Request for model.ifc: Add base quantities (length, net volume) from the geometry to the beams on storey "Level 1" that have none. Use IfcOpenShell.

First a look at what the model holds.

```python
import ifcopenshell
import ifcopenshell.util.element
import ifcopenshell.util.unit

model = ifcopenshell.open("model.ifc")
print(model.schema)
for unit_type in ("LENGTHUNIT", "AREAUNIT", "VOLUMEUNIT"):
    print(unit_type, ifcopenshell.util.unit.calculate_unit_scale(model, unit_type))
storey = next(s for s in model.by_type("IfcBuildingStorey") if s.Name == "Level 1")
beams = [e for e in ifcopenshell.util.element.get_decomposition(storey) if e.is_a("IfcBeam")]
for e in sorted(beams, key=lambda e: e.id()):
    print(e.id(), e.is_a(), e.Name, list(ifcopenshell.util.element.get_psets(e, qtos_only=True)), sep=" | ")
```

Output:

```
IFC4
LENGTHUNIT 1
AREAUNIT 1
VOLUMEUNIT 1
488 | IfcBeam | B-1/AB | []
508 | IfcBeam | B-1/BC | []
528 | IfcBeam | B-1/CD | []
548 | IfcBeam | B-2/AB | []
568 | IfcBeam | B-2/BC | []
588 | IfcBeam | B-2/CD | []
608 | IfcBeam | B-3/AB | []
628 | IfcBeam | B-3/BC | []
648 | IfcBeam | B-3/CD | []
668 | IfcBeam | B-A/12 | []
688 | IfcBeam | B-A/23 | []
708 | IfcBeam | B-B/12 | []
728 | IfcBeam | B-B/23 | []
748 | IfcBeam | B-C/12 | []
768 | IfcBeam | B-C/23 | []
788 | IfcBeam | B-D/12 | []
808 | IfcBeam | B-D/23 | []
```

```python
import ifcopenshell
import ifcopenshell.api.pset
import ifcopenshell.geom
import ifcopenshell.util.element
import ifcopenshell.util.shape
import ifcopenshell.util.unit

model = ifcopenshell.open("model.ifc")
unit_scale = ifcopenshell.util.unit.calculate_unit_scale(model)
volume_scale = ifcopenshell.util.unit.calculate_unit_scale(model, "VOLUMEUNIT")
settings = ifcopenshell.geom.settings()

storey = next(s for s in model.by_type("IfcBuildingStorey") if s.Name == "Level 1")
beams = [e for e in ifcopenshell.util.element.get_decomposition(storey) if e.is_a("IfcBeam")]

for e in sorted(beams, key=lambda e: e.id()):
    if ifcopenshell.util.element.get_psets(e, qtos_only=True, should_inherit=False):
        continue
    # Geometry comes back in metres, in the element's own axes.
    shape = ifcopenshell.geom.create_shape(settings, e)
    values = {
        "Length": ifcopenshell.util.shape.get_max_xyz(shape.geometry) / unit_scale,
        "NetVolume": ifcopenshell.util.shape.get_volume(shape.geometry) / volume_scale,
    }
    qto = ifcopenshell.api.pset.add_qto(model, product=e, name="Qto_BeamBaseQuantities")
    ifcopenshell.api.pset.edit_qto(model, qto=qto, properties=values)
    print(e.id(), {k: round(v, 3) for k, v in values.items()})

model.write("model_edited.ifc")
```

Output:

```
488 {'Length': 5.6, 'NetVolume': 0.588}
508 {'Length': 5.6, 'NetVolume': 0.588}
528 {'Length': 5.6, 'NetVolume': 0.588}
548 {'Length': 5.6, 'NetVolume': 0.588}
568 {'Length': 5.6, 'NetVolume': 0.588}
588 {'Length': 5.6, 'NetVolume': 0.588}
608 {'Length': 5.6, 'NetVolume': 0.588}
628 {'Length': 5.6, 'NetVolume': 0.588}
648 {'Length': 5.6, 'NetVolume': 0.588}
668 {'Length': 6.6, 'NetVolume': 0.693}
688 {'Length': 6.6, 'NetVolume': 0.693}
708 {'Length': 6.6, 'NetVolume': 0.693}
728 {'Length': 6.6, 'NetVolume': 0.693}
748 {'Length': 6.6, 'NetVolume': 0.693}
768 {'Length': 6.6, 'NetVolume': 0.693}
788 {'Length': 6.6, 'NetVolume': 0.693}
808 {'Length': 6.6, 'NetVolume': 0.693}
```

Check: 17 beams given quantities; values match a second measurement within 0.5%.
